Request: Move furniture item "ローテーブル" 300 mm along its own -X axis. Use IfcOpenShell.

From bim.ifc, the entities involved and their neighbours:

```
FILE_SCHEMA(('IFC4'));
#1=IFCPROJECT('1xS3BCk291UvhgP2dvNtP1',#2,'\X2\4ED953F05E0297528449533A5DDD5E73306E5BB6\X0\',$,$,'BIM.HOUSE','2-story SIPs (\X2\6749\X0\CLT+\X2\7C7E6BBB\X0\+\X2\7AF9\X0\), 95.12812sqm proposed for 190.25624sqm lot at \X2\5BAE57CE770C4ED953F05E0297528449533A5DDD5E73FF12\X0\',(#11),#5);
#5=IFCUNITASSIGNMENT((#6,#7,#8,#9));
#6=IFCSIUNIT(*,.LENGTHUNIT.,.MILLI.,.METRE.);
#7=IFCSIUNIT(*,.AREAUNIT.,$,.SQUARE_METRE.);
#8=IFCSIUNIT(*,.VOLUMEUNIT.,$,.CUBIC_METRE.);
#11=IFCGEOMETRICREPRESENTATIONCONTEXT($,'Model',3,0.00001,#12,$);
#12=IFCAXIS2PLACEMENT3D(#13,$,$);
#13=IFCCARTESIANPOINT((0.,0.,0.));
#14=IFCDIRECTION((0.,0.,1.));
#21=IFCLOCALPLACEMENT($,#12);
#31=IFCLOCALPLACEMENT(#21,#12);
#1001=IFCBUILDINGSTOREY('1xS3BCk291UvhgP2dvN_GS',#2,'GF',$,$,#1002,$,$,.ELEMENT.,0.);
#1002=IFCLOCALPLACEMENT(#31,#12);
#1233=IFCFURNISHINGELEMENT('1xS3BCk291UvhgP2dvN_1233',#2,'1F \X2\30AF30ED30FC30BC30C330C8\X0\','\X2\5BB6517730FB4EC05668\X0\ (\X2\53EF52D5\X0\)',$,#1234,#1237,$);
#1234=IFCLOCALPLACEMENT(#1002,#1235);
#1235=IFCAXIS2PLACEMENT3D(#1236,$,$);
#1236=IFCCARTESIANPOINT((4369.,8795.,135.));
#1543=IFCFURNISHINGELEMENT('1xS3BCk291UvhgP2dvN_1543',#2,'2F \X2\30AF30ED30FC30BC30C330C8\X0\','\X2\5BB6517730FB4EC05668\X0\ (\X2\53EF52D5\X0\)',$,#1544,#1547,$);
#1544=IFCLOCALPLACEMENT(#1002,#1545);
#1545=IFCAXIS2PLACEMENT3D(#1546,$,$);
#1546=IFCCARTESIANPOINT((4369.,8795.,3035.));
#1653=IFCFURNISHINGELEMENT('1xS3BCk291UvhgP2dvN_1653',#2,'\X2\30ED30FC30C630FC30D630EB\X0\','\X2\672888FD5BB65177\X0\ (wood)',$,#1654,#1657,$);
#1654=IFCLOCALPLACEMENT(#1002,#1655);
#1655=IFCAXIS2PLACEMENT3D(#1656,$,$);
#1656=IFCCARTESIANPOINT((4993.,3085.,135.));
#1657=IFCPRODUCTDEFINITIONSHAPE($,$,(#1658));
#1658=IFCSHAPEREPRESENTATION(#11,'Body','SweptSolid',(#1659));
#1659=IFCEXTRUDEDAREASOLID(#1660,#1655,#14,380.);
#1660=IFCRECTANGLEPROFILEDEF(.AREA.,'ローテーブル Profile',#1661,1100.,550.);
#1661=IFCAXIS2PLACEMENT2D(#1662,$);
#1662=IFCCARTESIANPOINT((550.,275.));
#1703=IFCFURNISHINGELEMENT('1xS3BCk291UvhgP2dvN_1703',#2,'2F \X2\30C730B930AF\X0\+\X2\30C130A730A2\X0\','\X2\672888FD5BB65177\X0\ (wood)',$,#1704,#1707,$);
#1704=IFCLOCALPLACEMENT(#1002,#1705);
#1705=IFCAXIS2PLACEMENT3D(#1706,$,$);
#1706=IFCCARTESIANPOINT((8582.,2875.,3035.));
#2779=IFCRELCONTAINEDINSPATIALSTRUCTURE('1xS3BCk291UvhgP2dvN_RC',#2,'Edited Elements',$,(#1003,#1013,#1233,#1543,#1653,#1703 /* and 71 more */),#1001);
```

```python
import ifcopenshell
import ifcopenshell.api.geometry
import ifcopenshell.util.placement
import ifcopenshell.util.unit

model = ifcopenshell.open("bim.ifc")
unit_scale = ifcopenshell.util.unit.calculate_unit_scale(model)

item = model.by_guid("1xS3BCk291UvhgP2dvN_1653")
matrix = ifcopenshell.util.placement.get_local_placement(item.ObjectPlacement)
matrix[:3, 3] -= matrix[:3, 0] * 0.3 / unit_scale
ifcopenshell.api.geometry.edit_object_placement(model, product=item, matrix=matrix, is_si=False)

print(ifcopenshell.util.placement.get_local_placement(item.ObjectPlacement).round(3) + 0.0)

model.write("bim_rev.ifc")
```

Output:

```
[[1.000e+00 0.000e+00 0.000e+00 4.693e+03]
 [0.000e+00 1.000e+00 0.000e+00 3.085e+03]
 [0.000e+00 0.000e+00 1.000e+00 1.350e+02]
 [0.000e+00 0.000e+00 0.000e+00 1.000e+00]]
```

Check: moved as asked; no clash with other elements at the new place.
